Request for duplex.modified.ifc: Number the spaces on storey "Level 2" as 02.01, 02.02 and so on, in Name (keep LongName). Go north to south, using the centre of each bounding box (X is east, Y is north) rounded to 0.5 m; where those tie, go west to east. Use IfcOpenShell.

First a look at what the model holds.

```python
import ifcopenshell
import ifcopenshell.util.element
import ifcopenshell.util.placement

model = ifcopenshell.open("duplex.modified.ifc")
print(model.schema)
storey = next(s for s in model.by_type("IfcBuildingStorey") if s.Name == "Level 2")
spaces = [e for e in ifcopenshell.util.element.get_decomposition(storey) if e.is_a("IfcSpace")]
for e in sorted(spaces, key=lambda e: e.id()):
    origin = ifcopenshell.util.placement.get_local_placement(e.ObjectPlacement)[:3, 3]
    print(e.id(), e.Name, e.LongName, origin.round(2) + 0.0, sep=" | ")
```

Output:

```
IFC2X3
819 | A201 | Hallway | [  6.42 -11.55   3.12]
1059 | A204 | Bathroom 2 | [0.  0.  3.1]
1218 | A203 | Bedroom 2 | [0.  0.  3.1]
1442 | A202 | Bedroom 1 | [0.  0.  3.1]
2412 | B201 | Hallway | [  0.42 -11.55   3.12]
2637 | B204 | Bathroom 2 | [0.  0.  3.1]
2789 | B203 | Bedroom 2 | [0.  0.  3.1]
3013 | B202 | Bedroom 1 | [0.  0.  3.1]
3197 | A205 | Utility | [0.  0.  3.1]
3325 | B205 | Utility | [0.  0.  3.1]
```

```python
import ifcopenshell
import ifcopenshell.geom
import ifcopenshell.util.element
import ifcopenshell.util.shape

model = ifcopenshell.open("duplex.modified.ifc")
settings = ifcopenshell.geom.settings()
settings.set("use-world-coords", True)


def centre(element):
    shape = ifcopenshell.geom.create_shape(settings, element)
    return ifcopenshell.util.shape.get_bbox_centroid(shape.geometry)


storey = next(s for s in model.by_type("IfcBuildingStorey") if s.Name == "Level 2")
spaces = [e for e in ifcopenshell.util.element.get_decomposition(storey) if e.is_a("IfcSpace")]

# Insertion points can sit at a corner or the storey origin, so sort by the geometry (in metres).
centres = {e: centre(e) for e in spaces}
spaces.sort(key=lambda e: (-round(centres[e][1] / 0.5), centres[e][0]))

for i, e in enumerate(spaces, start=1):
    number = f"02.{i:02d}"
    e.Name = number
    print(e.id(), number)

model.write("duplex.modified_updated.ifc")
```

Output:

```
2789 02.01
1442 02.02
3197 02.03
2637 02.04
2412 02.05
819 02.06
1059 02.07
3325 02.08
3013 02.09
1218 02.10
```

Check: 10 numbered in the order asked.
